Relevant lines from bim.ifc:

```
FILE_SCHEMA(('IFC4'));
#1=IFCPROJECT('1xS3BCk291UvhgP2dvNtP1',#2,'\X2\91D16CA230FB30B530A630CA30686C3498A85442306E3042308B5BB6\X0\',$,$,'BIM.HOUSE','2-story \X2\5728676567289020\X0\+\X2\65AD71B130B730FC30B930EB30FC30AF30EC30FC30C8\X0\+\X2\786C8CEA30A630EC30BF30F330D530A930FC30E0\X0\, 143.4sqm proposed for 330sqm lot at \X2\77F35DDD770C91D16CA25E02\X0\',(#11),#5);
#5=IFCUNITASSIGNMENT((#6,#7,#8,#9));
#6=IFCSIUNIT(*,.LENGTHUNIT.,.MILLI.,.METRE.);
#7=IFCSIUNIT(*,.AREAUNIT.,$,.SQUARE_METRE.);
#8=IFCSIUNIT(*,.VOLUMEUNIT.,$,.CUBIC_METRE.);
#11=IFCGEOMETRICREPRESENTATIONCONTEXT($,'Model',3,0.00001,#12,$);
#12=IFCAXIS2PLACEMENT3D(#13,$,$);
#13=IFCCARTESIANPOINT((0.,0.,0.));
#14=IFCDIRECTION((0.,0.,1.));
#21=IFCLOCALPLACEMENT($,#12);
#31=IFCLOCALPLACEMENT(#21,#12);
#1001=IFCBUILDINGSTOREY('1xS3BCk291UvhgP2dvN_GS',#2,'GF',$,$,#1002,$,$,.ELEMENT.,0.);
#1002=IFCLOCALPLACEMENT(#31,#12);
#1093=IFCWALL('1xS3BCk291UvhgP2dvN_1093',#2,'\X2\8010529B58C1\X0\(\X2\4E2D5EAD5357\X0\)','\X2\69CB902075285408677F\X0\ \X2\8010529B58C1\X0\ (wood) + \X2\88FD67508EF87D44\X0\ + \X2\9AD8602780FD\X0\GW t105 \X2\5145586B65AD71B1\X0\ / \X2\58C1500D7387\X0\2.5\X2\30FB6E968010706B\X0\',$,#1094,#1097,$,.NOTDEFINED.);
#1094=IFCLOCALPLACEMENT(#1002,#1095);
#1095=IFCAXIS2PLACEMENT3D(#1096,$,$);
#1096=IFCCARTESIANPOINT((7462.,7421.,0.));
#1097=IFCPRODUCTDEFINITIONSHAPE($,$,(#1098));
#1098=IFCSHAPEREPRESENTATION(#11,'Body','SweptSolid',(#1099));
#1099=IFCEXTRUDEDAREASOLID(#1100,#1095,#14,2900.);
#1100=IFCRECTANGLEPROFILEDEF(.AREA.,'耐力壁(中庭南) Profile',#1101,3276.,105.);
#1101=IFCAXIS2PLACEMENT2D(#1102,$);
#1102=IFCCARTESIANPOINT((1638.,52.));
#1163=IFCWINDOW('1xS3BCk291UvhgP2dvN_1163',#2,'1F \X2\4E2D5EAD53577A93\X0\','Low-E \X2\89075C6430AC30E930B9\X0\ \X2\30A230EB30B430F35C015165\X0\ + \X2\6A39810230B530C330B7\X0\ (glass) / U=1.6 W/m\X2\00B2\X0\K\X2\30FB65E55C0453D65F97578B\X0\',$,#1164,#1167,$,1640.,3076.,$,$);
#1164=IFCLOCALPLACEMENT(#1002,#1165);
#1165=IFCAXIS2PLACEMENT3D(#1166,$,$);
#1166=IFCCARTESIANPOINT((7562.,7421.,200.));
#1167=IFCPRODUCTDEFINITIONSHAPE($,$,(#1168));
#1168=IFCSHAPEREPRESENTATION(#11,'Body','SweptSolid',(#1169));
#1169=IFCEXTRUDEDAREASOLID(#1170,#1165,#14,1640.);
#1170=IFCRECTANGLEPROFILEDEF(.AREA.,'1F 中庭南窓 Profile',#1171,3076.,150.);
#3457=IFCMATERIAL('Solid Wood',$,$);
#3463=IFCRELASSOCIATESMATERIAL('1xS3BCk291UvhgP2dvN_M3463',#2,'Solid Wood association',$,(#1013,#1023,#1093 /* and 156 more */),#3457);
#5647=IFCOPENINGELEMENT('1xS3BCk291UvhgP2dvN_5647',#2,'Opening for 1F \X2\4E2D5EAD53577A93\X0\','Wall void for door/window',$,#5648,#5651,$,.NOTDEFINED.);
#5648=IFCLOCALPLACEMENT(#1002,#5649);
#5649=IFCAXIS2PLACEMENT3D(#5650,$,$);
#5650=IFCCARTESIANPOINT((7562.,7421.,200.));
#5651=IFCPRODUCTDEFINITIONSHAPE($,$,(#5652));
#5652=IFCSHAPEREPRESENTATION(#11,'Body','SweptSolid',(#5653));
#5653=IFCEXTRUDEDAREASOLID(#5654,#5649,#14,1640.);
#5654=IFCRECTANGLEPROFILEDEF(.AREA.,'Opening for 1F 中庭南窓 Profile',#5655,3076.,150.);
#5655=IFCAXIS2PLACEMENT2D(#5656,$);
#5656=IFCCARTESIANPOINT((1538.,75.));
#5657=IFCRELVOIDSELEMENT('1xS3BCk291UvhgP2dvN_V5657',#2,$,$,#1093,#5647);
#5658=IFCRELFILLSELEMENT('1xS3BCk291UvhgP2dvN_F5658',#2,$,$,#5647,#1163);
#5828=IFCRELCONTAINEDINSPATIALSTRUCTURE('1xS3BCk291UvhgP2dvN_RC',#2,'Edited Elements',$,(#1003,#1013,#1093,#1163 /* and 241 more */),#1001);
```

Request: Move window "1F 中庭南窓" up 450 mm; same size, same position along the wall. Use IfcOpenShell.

```python
import numpy as np
import ifcopenshell
import ifcopenshell.api.geometry
import ifcopenshell.util.placement
import ifcopenshell.util.unit

model = ifcopenshell.open("bim.ifc")
unit_scale = ifcopenshell.util.unit.calculate_unit_scale(model)

window = model.by_id(1163)
opening = window.FillsVoids[0].RelatingOpeningElement
dz = 0.45 / unit_scale

shift = np.array([0.0, 0.0, dz])
# The window is not placed relative to its opening, so move both.
for product in (opening, window):
    matrix = ifcopenshell.util.placement.get_local_placement(product.ObjectPlacement)
    matrix[:3, 3] += shift
    ifcopenshell.api.geometry.edit_object_placement(model, product=product, matrix=matrix, is_si=False)

print(f"moved by {dz * unit_scale:+.3f} m")

model.write("bim_edited.ifc")
```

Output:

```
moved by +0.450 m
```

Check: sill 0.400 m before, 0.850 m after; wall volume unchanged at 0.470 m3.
